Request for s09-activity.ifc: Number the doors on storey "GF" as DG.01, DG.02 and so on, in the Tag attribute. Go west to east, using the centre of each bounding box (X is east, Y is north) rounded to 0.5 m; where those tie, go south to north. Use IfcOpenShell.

First a look at what the model holds.

```python
import ifcopenshell
import ifcopenshell.util.element
import ifcopenshell.util.placement

model = ifcopenshell.open("s09-activity.ifc")
print(model.schema)
storey = next(s for s in model.by_type("IfcBuildingStorey") if s.Name == "GF")
doors = [e for e in ifcopenshell.util.element.get_decomposition(storey) if e.is_a("IfcDoor")]
for e in sorted(doors, key=lambda e: e.id()):
    origin = ifcopenshell.util.placement.get_local_placement(e.ObjectPlacement)[:3, 3]
    print(e.id(), e.Tag, e.Name, origin.round(2) + 0.0, sep=" | ")
```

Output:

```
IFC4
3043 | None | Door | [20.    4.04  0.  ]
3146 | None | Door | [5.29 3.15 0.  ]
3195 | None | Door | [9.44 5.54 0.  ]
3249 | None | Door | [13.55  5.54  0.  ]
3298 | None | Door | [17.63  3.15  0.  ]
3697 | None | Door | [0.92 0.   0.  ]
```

```python
import ifcopenshell
import ifcopenshell.geom
import ifcopenshell.util.element
import ifcopenshell.util.shape

model = ifcopenshell.open("s09-activity.ifc")
settings = ifcopenshell.geom.settings()
settings.set("use-world-coords", True)


def centre(element):
    shape = ifcopenshell.geom.create_shape(settings, element)
    return ifcopenshell.util.shape.get_bbox_centroid(shape.geometry)


storey = next(s for s in model.by_type("IfcBuildingStorey") if s.Name == "GF")
doors = [e for e in ifcopenshell.util.element.get_decomposition(storey) if e.is_a("IfcDoor")]

# Insertion points can sit at a corner or the storey origin, so sort by the geometry (in metres).
centres = {e: centre(e) for e in doors}
doors.sort(key=lambda e: (round(centres[e][0] / 0.5), centres[e][1]))

for i, e in enumerate(doors, start=1):
    number = f"DG.{i:02d}"
    e.Tag = number
    print(e.id(), number)

model.write("s09-activity-out.ifc")
```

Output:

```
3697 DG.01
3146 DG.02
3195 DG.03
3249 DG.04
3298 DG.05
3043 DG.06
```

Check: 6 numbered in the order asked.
